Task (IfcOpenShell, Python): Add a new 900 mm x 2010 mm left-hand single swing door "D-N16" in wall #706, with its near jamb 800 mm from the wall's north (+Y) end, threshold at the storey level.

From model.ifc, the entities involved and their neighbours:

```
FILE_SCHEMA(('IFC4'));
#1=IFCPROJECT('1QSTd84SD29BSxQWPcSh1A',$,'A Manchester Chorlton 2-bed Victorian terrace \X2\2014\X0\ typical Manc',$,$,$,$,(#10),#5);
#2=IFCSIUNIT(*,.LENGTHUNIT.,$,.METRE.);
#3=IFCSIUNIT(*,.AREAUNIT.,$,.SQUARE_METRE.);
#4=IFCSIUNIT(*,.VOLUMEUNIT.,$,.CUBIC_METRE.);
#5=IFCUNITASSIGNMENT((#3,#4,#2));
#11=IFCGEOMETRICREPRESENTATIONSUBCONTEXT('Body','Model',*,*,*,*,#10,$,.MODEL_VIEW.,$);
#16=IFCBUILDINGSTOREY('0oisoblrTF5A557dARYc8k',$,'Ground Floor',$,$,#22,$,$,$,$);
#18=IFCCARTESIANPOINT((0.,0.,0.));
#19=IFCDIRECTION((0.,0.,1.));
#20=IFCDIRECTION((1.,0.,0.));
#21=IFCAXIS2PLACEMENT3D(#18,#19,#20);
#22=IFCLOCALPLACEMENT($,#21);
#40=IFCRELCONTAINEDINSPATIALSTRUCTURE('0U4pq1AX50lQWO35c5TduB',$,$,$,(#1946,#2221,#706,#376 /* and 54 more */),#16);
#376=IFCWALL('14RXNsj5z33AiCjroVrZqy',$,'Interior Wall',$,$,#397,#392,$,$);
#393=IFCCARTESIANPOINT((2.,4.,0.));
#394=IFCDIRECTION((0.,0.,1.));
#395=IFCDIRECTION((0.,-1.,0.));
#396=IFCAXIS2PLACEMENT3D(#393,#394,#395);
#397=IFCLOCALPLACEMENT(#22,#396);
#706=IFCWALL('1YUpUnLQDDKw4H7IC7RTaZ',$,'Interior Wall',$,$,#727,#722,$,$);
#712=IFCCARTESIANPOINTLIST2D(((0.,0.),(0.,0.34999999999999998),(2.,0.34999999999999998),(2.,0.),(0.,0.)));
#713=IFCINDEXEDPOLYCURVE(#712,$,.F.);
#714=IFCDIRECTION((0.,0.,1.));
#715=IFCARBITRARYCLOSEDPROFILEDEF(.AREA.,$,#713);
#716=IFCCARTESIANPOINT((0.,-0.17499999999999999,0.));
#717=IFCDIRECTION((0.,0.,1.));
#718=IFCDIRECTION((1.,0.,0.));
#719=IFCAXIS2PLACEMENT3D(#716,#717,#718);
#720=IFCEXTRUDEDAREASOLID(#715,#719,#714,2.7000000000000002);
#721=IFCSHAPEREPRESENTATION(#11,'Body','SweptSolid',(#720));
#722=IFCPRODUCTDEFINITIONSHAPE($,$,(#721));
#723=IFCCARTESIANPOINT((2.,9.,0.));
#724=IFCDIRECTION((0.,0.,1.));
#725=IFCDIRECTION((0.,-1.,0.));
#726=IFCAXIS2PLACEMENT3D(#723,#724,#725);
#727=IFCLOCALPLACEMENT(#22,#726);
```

```python
import numpy as np
import ifcopenshell
import ifcopenshell.api.feature
import ifcopenshell.api.geometry
import ifcopenshell.api.root
import ifcopenshell.api.spatial
import ifcopenshell.geom
import ifcopenshell.util.element
import ifcopenshell.util.placement
import ifcopenshell.util.representation
import ifcopenshell.util.shape
import ifcopenshell.util.unit

model = ifcopenshell.open("model.ifc")
unit_scale = ifcopenshell.util.unit.calculate_unit_scale(model)
settings = ifcopenshell.geom.settings()


def volume(element):
    """Net volume in cubic metres, openings subtracted."""
    shape = ifcopenshell.geom.create_shape(settings, element)
    return ifcopenshell.util.shape.get_volume(shape.geometry)


wall = model.by_id(706)
storey = ifcopenshell.util.element.get_container(wall, ifc_class="IfcBuildingStorey")
context = ifcopenshell.util.representation.get_context(model, "Model", "Body", "MODEL_VIEW")
before = volume(wall)

width, height, from_end, sill = 0.9, 2.01, 0.8, 0.0  # metres

# The wall runs along its own X axis, and the end named is its -X end.
wall_shape = ifcopenshell.geom.create_shape(settings, wall)
x, y, z = ifcopenshell.util.shape.get_vertices(wall_shape.geometry).T
start = x.min() + from_end
face, thickness = float(y.min()), float(y.max() - y.min())
wall_matrix = ifcopenshell.util.placement.get_local_placement(wall.ObjectPlacement)
level = ifcopenshell.util.placement.get_local_placement(storey.ObjectPlacement)[2, 3]


def in_wall(x, y):
    """Placement at x, y metres in the wall's axes, at sill height."""
    matrix = wall_matrix.copy()
    matrix[:, 3] = wall_matrix @ np.array([x / unit_scale, y / unit_scale, 0.0, 1.0])
    matrix[2, 3] = level + sill / unit_scale
    return matrix


# Opening: a box that overshoots both wall faces by 50 mm.
opening = ifcopenshell.api.root.create_entity(model, ifc_class="IfcOpeningElement", predefined_type="OPENING")
box = ifcopenshell.api.geometry.add_wall_representation(
    model, context=context, length=width, height=height, thickness=thickness + 0.1
)
ifcopenshell.api.geometry.assign_representation(model, product=opening, representation=box)
ifcopenshell.api.geometry.edit_object_placement(model, product=opening, matrix=in_wall(start, face - 0.05), is_si=False)
ifcopenshell.api.feature.add_feature(model, feature=opening, element=wall)

door = ifcopenshell.api.root.create_entity(model, ifc_class="IfcDoor", name="D-N16", predefined_type="DOOR")
door.OverallWidth, door.OverallHeight = width / unit_scale, height / unit_scale
door.OperationType = "SINGLE_SWING_LEFT"
body = ifcopenshell.api.geometry.add_door_representation(
    model,
    context=context,
    overall_width=door.OverallWidth,
    overall_height=door.OverallHeight,
    operation_type="SINGLE_SWING_LEFT",
    lining_properties={"LiningDepth": thickness / unit_scale, "ThresholdDepth": thickness / unit_scale},
)
ifcopenshell.api.geometry.assign_representation(model, product=door, representation=body)
ifcopenshell.api.spatial.assign_container(model, products=[door], relating_structure=storey)
ifcopenshell.api.feature.add_filling(model, opening=opening, element=door)

# The lining spans the wall, so the door starts at the wall face.
ifcopenshell.api.geometry.edit_object_placement(model, product=door, matrix=in_wall(start, face), is_si=False)

after = volume(wall)

print(f"wall volume {before:.3f} -> {after:.3f} m3")

model.write("model_rev.ifc")
```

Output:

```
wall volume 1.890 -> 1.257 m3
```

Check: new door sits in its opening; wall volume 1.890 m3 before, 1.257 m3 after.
